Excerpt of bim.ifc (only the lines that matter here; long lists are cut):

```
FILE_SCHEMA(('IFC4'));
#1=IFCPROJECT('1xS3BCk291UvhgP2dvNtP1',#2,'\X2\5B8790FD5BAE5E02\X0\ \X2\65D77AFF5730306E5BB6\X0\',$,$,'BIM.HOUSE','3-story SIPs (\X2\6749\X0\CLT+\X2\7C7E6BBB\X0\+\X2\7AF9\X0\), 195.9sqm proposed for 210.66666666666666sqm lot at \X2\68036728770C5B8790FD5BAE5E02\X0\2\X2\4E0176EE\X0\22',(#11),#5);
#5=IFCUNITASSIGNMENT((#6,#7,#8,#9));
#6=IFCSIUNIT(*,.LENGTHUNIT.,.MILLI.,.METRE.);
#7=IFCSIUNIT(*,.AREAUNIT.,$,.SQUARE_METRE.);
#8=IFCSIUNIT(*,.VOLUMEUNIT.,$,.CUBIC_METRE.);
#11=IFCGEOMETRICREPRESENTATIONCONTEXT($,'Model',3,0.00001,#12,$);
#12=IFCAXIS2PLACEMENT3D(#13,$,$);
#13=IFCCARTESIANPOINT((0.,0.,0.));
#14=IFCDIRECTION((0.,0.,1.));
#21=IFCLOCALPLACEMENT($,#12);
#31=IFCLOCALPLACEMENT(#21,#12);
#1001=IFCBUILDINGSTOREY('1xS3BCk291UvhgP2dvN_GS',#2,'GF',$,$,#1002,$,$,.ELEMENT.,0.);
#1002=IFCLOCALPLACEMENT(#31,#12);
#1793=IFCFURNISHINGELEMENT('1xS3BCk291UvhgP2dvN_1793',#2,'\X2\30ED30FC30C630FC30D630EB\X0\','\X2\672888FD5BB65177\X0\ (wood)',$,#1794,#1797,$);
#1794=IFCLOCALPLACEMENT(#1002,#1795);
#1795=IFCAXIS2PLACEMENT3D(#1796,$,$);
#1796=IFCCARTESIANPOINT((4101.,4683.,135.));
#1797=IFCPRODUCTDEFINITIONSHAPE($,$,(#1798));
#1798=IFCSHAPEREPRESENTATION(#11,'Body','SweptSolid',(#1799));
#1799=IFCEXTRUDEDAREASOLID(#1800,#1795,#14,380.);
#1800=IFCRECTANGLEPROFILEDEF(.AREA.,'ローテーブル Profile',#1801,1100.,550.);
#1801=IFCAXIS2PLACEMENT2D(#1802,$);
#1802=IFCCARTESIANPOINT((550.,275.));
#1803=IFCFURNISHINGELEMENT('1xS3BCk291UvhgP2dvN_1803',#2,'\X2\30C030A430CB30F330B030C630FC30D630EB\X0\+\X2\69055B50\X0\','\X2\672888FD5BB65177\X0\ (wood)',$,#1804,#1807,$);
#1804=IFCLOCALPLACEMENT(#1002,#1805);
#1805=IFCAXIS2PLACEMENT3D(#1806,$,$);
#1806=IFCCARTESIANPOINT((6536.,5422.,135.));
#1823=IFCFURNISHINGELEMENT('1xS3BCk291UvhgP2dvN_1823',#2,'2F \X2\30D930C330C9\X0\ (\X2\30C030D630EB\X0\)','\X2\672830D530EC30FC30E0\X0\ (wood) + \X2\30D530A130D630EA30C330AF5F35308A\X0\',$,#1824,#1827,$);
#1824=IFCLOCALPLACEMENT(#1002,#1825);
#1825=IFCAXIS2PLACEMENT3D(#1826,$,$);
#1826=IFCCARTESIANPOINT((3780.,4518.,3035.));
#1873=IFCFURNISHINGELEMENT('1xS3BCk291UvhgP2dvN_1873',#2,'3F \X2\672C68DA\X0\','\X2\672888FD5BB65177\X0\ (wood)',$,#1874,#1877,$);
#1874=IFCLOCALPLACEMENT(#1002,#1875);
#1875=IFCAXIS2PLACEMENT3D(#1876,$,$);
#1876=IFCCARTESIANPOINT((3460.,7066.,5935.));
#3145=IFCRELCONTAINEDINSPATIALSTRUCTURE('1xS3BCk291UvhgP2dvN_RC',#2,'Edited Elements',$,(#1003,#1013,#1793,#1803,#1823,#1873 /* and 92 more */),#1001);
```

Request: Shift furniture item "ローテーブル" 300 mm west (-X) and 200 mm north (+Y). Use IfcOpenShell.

```python
import ifcopenshell
import ifcopenshell.api.geometry
import ifcopenshell.util.placement

model = ifcopenshell.open("bim.ifc")

item = model.by_id(1793)
matrix = ifcopenshell.util.placement.get_local_placement(item.ObjectPlacement)
matrix[0, 3] -= 300.0
matrix[1, 3] += 200.0
ifcopenshell.api.geometry.edit_object_placement(model, product=item, matrix=matrix, is_si=False)

print(ifcopenshell.util.placement.get_local_placement(item.ObjectPlacement).round(3) + 0.0)

model.write("bim-out.ifc")
```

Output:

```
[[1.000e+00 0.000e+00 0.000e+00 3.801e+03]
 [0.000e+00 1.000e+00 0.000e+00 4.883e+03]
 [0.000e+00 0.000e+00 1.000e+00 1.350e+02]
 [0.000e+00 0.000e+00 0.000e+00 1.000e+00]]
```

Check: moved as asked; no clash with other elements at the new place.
